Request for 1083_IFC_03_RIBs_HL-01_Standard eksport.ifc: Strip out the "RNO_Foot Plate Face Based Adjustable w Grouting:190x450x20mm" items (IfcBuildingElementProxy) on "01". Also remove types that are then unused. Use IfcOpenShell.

First a look at what the model holds.

```python
import ifcopenshell
import ifcopenshell.util.element

model = ifcopenshell.open("1083_IFC_03_RIBs_HL-01_Standard eksport.ifc")
print(model.schema)
storey = next(s for s in model.by_type("IfcBuildingStorey") if s.Name == "01")
proxies = [e for e in ifcopenshell.util.element.get_decomposition(storey) if e.is_a("IfcBuildingElementProxy")]
seen = {}
for e in proxies:
    element_type = ifcopenshell.util.element.get_type(e)
    name = element_type.Name if element_type not in (None, e) else None
    seen[name] = seen.get(name, 0) + 1
for name, count in sorted(seen.items(), key=str):
    print(count, "x", name)
```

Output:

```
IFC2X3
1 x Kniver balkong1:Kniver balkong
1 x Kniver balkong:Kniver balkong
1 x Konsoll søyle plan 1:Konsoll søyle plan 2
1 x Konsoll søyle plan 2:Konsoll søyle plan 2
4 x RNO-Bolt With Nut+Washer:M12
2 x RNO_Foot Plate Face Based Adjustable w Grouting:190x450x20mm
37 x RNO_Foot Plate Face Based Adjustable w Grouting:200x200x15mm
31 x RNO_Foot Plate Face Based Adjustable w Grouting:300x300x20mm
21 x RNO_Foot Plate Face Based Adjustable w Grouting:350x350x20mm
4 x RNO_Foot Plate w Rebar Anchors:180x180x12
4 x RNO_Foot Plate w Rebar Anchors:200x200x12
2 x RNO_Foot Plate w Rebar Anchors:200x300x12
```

```python
import ifcopenshell
import ifcopenshell.api.root
import ifcopenshell.util.element

model = ifcopenshell.open("1083_IFC_03_RIBs_HL-01_Standard eksport.ifc")

storey = next(s for s in model.by_type("IfcBuildingStorey") if s.Name == "01")
proxies = [e for e in ifcopenshell.util.element.get_decomposition(storey) if e.is_a("IfcBuildingElementProxy")]
targets = [e for e in proxies if (t := ifcopenshell.util.element.get_type(e)) not in (None, e) and t.Name == "RNO_Foot Plate Face Based Adjustable w Grouting:190x450x20mm"]
types = {ifcopenshell.util.element.get_type(e) for e in targets} - {None, *targets}

for e in targets:
    ifcopenshell.api.root.remove_product(model, product=e)
print(len(targets), "removed")

unused = [t for t in types if not ifcopenshell.util.element.get_types(t)]
for t in unused:
    ifcopenshell.api.root.remove_product(model, product=t)
print(len(unused), "unused types removed")

model.write("1083_IFC_03_RIBs_HL-01_Standard eksport_edited.ifc")
```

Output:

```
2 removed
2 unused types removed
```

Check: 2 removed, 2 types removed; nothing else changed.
